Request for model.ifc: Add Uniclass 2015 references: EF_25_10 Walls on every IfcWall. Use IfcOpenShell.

First a look at what the model holds.

```python
import ifcopenshell

model = ifcopenshell.open("model.ifc")
print(model.schema)
print("classifications:", [c.Name for c in model.by_type("IfcClassification")])
for ifc_class in ("IfcDoor", "IfcRoof", "IfcStair", "IfcWall", "IfcWindow"):
    print(ifc_class, len(model.by_type(ifc_class)))
```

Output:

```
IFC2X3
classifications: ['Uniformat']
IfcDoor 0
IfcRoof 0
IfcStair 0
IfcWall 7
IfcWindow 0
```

```python
import ifcopenshell
import ifcopenshell.api.classification

model = ifcopenshell.open("model.ifc")

# IFC2X3 requires Source and Edition and has no link from the project to the system.
system = model.create_entity("IfcClassification", Source="NBS", Edition="2015", Name="Uniclass 2015")

codes = {
    "IfcWall": ("EF_25_10", "Walls"),
}
for ifc_class, (code, name) in codes.items():
    products = model.by_type(ifc_class)
    ifcopenshell.api.classification.add_reference(
        model, products=products, classification=system, identification=code, name=name
    )
    print(code, len(products))

model.write("model_updated.ifc")
```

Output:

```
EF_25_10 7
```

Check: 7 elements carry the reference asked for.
